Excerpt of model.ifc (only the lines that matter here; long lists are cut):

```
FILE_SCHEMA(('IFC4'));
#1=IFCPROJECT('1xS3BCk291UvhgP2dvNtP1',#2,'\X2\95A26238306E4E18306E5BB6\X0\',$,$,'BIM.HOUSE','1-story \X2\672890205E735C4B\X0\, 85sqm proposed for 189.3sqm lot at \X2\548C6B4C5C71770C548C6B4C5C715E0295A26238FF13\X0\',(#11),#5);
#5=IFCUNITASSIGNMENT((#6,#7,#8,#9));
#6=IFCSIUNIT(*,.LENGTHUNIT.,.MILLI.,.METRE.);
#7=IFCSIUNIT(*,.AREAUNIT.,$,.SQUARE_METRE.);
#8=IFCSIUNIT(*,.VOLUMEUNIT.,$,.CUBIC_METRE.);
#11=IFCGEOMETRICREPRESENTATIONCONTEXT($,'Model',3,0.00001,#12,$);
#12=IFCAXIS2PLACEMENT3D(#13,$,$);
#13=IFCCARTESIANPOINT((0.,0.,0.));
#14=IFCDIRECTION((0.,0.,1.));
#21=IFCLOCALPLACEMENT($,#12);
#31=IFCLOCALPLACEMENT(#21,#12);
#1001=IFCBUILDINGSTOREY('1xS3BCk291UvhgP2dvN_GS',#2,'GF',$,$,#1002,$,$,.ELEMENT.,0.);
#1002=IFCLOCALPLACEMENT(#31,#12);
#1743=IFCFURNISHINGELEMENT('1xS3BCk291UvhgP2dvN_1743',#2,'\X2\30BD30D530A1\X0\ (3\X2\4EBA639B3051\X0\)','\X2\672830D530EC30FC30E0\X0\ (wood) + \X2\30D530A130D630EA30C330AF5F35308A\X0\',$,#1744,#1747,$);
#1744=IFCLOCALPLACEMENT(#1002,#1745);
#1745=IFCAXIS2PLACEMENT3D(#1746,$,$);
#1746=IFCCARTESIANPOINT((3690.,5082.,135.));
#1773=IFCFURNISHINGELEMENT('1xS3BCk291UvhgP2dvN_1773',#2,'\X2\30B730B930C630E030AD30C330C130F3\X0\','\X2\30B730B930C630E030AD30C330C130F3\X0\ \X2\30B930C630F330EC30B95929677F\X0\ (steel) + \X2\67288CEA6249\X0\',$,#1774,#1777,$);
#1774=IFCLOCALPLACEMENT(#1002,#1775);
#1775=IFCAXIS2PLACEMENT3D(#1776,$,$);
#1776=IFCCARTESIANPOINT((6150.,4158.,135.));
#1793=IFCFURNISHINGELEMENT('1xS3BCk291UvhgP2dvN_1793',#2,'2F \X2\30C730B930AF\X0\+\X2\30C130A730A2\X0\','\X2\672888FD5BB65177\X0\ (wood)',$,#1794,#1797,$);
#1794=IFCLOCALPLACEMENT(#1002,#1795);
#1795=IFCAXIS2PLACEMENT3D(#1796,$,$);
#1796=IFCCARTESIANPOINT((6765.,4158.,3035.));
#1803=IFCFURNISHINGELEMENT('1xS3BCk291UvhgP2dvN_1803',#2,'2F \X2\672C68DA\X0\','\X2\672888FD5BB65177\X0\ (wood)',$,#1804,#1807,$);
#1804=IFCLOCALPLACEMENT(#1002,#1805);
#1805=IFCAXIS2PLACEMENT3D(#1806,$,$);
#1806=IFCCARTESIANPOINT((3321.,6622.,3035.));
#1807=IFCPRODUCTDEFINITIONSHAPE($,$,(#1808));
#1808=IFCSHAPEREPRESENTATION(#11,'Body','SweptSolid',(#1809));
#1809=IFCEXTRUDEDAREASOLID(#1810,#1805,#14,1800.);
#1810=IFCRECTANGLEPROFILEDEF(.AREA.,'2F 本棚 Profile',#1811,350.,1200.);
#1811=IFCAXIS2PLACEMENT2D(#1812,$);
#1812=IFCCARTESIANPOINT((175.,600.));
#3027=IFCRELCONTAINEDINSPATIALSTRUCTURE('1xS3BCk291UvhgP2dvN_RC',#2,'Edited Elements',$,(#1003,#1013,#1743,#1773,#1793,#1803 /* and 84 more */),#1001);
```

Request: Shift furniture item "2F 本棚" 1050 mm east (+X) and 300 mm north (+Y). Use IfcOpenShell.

```python
import ifcopenshell
import ifcopenshell.api.geometry
import ifcopenshell.util.placement
import ifcopenshell.util.unit

model = ifcopenshell.open("model.ifc")
unit_scale = ifcopenshell.util.unit.calculate_unit_scale(model)

item = model.by_guid("1xS3BCk291UvhgP2dvN_1803")
matrix = ifcopenshell.util.placement.get_local_placement(item.ObjectPlacement)
matrix[0, 3] += 1.05 / unit_scale
matrix[1, 3] += 0.3 / unit_scale
ifcopenshell.api.geometry.edit_object_placement(model, product=item, matrix=matrix, is_si=False)

print(ifcopenshell.util.placement.get_local_placement(item.ObjectPlacement).round(3) + 0.0)

model.write("model_rev.ifc")
```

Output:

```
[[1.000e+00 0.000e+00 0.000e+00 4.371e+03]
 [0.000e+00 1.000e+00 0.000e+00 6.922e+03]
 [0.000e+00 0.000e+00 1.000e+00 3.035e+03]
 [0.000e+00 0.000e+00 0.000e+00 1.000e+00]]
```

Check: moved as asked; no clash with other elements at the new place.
